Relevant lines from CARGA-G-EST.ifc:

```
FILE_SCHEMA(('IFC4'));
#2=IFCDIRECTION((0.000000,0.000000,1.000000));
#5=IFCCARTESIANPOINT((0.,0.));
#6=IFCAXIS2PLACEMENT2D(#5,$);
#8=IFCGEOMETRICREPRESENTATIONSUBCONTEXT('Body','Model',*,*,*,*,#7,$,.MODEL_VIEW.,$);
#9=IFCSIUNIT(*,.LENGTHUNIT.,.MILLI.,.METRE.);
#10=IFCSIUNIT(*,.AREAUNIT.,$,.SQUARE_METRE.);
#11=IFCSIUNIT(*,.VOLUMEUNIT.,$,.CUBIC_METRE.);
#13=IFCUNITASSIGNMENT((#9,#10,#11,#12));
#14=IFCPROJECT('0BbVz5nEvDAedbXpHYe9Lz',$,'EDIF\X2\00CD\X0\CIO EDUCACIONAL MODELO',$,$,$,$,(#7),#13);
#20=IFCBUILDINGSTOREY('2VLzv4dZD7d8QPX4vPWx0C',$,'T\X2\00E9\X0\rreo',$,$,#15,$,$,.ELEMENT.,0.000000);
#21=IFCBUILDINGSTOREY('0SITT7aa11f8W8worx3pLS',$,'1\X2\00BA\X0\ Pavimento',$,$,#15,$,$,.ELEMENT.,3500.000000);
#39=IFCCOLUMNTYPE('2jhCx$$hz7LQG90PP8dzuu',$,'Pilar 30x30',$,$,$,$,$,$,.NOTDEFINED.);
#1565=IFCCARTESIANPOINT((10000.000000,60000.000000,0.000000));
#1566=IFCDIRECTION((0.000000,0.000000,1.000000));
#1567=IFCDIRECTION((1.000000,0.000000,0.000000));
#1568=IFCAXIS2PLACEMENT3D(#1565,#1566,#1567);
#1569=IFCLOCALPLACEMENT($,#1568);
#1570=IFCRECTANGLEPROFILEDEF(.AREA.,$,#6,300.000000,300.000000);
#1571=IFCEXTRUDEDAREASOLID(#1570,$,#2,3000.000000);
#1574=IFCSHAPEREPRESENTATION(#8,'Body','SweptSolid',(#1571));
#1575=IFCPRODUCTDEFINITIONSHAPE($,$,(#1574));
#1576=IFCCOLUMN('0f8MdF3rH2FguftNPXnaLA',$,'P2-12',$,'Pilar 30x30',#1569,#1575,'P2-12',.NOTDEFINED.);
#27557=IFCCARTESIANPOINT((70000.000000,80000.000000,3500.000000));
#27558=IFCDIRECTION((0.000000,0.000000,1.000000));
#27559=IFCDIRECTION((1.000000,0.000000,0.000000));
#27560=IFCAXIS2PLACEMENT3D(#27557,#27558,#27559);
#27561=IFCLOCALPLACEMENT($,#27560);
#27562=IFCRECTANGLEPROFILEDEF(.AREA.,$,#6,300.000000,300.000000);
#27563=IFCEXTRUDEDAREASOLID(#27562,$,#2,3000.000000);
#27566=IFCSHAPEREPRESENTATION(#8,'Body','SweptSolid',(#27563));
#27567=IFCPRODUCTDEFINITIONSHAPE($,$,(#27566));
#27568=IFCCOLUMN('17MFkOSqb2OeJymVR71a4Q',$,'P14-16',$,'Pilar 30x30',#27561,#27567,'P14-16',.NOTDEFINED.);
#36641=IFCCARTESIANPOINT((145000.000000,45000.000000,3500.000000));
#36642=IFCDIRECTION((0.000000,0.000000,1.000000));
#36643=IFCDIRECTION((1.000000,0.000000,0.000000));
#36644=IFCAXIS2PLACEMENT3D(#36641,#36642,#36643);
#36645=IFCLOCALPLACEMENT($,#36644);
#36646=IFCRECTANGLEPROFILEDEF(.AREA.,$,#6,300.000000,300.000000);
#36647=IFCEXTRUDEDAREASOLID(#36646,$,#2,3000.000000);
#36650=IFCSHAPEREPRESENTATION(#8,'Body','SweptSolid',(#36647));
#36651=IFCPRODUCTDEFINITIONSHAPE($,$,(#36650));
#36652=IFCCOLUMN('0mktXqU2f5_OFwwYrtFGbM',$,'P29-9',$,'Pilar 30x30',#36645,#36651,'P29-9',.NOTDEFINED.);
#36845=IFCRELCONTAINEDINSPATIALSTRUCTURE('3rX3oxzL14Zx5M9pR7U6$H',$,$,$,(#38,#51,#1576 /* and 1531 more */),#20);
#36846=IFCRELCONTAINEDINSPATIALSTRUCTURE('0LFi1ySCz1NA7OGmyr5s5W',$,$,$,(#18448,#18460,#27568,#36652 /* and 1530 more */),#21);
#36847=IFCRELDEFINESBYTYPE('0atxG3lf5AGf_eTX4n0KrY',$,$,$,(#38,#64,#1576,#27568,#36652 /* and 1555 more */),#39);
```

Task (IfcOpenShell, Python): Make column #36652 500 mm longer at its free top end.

```python
import ifcopenshell
import ifcopenshell.util.representation

model = ifcopenshell.open("CARGA-G-EST.ifc")

member = model.by_guid("0mktXqU2f5_OFwwYrtFGbM")
change = 500.0

# The extrusion runs towards the end named, so only its depth changes.
body = ifcopenshell.util.representation.get_representation(member, "Model", "Body")
solid = body.Items[0]
old_length = solid.Depth
solid.Depth += change

print(f"length {old_length:g} -> {solid.Depth:g}")

model.write("CARGA-G-EST_edited.ifc")
```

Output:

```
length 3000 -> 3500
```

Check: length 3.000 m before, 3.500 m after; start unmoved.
